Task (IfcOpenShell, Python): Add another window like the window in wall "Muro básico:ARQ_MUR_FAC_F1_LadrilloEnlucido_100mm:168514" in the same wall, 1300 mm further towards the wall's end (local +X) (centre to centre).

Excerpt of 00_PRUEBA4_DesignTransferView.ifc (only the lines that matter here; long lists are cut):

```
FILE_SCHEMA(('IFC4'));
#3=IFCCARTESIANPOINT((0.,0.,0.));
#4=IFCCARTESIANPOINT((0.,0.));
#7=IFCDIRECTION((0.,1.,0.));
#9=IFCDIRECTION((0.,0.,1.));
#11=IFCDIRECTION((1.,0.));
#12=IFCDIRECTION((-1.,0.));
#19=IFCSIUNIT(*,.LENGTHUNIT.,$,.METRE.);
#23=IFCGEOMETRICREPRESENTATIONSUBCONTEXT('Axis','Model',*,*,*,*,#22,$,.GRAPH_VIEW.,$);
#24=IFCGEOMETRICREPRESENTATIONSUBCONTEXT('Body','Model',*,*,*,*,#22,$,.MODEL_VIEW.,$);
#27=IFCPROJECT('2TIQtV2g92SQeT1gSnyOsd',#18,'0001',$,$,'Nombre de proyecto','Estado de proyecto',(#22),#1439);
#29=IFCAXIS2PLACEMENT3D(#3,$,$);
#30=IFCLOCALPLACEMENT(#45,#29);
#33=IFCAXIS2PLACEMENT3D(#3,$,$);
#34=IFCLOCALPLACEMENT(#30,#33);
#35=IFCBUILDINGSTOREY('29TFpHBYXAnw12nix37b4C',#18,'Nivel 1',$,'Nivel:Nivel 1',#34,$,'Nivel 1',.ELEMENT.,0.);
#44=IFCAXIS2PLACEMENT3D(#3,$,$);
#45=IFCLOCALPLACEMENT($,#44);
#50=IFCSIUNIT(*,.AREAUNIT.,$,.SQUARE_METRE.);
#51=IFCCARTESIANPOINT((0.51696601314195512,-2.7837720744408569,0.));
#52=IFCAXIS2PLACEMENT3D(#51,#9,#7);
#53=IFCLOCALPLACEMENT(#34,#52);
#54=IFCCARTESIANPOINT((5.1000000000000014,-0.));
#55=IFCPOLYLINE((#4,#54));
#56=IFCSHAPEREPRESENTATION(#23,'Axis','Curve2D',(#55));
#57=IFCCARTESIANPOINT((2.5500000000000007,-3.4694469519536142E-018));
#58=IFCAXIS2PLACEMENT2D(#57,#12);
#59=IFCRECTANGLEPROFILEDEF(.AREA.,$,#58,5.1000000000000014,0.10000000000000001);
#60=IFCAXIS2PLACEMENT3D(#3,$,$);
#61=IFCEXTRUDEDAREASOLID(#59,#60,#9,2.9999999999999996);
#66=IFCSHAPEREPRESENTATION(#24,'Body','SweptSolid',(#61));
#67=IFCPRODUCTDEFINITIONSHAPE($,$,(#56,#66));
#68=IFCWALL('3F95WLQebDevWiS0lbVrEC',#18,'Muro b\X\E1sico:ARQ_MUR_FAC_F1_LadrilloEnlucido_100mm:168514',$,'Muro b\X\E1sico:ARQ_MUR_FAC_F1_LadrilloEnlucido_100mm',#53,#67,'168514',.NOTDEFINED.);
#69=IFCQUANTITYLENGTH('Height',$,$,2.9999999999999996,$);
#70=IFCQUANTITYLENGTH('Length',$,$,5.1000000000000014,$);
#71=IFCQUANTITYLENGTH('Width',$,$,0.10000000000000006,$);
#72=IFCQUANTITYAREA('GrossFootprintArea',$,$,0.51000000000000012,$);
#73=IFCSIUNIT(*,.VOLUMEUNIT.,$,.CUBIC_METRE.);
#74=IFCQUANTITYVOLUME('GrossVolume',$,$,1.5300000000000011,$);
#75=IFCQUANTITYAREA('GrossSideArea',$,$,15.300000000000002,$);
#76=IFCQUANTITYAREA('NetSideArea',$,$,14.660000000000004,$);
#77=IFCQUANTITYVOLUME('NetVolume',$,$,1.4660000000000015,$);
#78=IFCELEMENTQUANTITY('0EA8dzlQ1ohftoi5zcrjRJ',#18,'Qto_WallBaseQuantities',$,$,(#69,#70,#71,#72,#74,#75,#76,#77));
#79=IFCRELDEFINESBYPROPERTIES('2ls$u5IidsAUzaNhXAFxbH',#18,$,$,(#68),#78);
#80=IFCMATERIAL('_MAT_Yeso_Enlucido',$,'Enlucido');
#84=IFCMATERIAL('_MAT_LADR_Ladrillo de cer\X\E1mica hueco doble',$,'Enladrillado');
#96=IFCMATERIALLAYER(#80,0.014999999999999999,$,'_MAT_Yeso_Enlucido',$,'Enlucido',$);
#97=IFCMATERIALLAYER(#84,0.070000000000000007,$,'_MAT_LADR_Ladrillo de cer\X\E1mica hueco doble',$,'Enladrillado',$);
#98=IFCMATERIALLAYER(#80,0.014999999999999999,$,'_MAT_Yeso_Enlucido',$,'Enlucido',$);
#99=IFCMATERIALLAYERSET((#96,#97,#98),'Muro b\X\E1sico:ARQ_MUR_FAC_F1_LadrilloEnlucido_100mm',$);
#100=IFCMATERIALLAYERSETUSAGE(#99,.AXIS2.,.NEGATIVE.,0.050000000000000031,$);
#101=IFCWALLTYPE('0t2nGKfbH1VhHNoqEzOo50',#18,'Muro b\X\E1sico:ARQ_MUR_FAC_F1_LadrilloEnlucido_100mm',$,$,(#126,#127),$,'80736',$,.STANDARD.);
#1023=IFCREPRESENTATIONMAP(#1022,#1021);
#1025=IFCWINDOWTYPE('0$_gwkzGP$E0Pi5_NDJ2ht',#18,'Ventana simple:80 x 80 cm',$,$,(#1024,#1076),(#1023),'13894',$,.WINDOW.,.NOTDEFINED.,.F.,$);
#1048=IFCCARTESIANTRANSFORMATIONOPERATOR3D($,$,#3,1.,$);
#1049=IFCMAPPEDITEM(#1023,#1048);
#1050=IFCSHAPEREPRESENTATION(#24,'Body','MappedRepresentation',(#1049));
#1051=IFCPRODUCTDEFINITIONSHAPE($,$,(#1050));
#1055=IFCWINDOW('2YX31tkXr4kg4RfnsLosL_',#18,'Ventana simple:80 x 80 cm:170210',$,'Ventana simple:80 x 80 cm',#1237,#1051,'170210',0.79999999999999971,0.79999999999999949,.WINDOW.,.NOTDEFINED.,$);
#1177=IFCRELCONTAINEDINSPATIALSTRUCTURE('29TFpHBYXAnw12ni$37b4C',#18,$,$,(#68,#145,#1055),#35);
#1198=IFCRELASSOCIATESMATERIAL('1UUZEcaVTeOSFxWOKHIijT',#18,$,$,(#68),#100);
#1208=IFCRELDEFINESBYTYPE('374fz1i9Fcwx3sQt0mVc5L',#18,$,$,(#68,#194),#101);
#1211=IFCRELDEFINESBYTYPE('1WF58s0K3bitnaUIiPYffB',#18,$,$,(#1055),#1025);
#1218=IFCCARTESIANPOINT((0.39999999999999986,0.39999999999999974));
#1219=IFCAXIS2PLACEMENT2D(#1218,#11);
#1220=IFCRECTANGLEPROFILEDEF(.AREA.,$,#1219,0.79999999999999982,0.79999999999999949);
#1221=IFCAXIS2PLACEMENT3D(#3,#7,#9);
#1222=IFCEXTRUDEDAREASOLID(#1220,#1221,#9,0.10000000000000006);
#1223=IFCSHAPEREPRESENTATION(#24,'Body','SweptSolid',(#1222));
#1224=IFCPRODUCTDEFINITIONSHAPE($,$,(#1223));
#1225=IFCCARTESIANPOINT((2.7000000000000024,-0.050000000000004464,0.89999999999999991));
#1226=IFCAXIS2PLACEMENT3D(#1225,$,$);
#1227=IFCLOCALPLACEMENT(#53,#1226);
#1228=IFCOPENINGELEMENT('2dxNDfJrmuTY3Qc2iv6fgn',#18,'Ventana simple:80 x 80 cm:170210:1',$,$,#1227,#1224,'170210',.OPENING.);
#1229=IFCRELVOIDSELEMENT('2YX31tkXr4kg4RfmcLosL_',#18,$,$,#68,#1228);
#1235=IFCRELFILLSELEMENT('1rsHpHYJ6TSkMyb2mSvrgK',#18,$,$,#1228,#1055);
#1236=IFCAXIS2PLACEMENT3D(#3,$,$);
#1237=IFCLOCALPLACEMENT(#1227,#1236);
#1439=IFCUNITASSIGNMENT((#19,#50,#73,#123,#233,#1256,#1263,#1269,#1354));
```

```python
import ifcopenshell
import ifcopenshell.api.feature
import ifcopenshell.api.geometry
import ifcopenshell.api.pset
import ifcopenshell.api.root
import ifcopenshell.geom
import ifcopenshell.util.element
import ifcopenshell.util.placement
import ifcopenshell.util.shape
import ifcopenshell.util.unit

model = ifcopenshell.open("00_PRUEBA4_DesignTransferView.ifc")
unit_scale = ifcopenshell.util.unit.calculate_unit_scale(model)
area_scale = ifcopenshell.util.unit.calculate_unit_scale(model, "AREAUNIT")
volume_scale = ifcopenshell.util.unit.calculate_unit_scale(model, "VOLUMEUNIT")
settings = ifcopenshell.geom.settings()


def volume(element):
    """Net volume in cubic metres, openings subtracted."""
    shape = ifcopenshell.geom.create_shape(settings, element)
    return ifcopenshell.util.shape.get_volume(shape.geometry)


def reuse_history(source, copy):
    """copy_class also copies each property set's owner history, people and application; keep the originals."""
    for rel in copy.IsDefinedBy:
        if rel.is_a("IfcRelDefinesByProperties") and (history := rel.RelatingPropertyDefinition.OwnerHistory):
            rel.RelatingPropertyDefinition.OwnerHistory = source.OwnerHistory
            ifcopenshell.util.element.remove_deep2(model, history)


window = model.by_id(1055)
opening = window.FillsVoids[0].RelatingOpeningElement
wall = opening.VoidsElements[0].RelatingBuildingElement
before = volume(wall)
shift = ifcopenshell.util.placement.get_local_placement(wall.ObjectPlacement)[:3, 0] * 1.3 / unit_scale

# copy_class copies the void relationship, type, container and properties, but no geometry.
new_opening = ifcopenshell.api.root.copy_class(model, product=opening)
new_opening.Representation = ifcopenshell.util.element.copy_deep(
    model, opening.Representation, exclude=["IfcGeometricRepresentationContext", "IfcRepresentationMap"]
)
new_opening.Name = "Ventana simple:80 x 80 cm"
new_opening.Tag = None
reuse_history(opening, new_opening)
new_window = ifcopenshell.api.root.copy_class(model, product=window)
new_window.Representation = ifcopenshell.util.element.copy_deep(
    model, window.Representation, exclude=["IfcGeometricRepresentationContext", "IfcRepresentationMap"]
)
new_window.Name = "Ventana simple:80 x 80 cm"
new_window.Tag = None
reuse_history(window, new_window)
ifcopenshell.api.feature.add_filling(model, opening=new_opening, element=new_window)

for old, new in ((opening, new_opening), (window, new_window)):
    matrix = ifcopenshell.util.placement.get_local_placement(old.ObjectPlacement)
    matrix[:3, 3] += shift
    ifcopenshell.api.geometry.edit_object_placement(model, product=new, matrix=matrix, is_si=False)

after = volume(wall)
thickness = 0.1  # wall thickness in metres

# Update the wall's stored quantities.
qto = model.by_id(ifcopenshell.util.element.get_pset(wall, "Qto_WallBaseQuantities", should_inherit=False)["id"])
ifcopenshell.api.pset.edit_qto(model, qto=qto, properties={
    "NetSideArea": after / thickness / area_scale,
    "NetVolume": after / volume_scale,
})

print(f"wall volume {before:.3f} -> {after:.3f} m3")

model.write("00_PRUEBA4_DesignTransferView-out.ifc")
```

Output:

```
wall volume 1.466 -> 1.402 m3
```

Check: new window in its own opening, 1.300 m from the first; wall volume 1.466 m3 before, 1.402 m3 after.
